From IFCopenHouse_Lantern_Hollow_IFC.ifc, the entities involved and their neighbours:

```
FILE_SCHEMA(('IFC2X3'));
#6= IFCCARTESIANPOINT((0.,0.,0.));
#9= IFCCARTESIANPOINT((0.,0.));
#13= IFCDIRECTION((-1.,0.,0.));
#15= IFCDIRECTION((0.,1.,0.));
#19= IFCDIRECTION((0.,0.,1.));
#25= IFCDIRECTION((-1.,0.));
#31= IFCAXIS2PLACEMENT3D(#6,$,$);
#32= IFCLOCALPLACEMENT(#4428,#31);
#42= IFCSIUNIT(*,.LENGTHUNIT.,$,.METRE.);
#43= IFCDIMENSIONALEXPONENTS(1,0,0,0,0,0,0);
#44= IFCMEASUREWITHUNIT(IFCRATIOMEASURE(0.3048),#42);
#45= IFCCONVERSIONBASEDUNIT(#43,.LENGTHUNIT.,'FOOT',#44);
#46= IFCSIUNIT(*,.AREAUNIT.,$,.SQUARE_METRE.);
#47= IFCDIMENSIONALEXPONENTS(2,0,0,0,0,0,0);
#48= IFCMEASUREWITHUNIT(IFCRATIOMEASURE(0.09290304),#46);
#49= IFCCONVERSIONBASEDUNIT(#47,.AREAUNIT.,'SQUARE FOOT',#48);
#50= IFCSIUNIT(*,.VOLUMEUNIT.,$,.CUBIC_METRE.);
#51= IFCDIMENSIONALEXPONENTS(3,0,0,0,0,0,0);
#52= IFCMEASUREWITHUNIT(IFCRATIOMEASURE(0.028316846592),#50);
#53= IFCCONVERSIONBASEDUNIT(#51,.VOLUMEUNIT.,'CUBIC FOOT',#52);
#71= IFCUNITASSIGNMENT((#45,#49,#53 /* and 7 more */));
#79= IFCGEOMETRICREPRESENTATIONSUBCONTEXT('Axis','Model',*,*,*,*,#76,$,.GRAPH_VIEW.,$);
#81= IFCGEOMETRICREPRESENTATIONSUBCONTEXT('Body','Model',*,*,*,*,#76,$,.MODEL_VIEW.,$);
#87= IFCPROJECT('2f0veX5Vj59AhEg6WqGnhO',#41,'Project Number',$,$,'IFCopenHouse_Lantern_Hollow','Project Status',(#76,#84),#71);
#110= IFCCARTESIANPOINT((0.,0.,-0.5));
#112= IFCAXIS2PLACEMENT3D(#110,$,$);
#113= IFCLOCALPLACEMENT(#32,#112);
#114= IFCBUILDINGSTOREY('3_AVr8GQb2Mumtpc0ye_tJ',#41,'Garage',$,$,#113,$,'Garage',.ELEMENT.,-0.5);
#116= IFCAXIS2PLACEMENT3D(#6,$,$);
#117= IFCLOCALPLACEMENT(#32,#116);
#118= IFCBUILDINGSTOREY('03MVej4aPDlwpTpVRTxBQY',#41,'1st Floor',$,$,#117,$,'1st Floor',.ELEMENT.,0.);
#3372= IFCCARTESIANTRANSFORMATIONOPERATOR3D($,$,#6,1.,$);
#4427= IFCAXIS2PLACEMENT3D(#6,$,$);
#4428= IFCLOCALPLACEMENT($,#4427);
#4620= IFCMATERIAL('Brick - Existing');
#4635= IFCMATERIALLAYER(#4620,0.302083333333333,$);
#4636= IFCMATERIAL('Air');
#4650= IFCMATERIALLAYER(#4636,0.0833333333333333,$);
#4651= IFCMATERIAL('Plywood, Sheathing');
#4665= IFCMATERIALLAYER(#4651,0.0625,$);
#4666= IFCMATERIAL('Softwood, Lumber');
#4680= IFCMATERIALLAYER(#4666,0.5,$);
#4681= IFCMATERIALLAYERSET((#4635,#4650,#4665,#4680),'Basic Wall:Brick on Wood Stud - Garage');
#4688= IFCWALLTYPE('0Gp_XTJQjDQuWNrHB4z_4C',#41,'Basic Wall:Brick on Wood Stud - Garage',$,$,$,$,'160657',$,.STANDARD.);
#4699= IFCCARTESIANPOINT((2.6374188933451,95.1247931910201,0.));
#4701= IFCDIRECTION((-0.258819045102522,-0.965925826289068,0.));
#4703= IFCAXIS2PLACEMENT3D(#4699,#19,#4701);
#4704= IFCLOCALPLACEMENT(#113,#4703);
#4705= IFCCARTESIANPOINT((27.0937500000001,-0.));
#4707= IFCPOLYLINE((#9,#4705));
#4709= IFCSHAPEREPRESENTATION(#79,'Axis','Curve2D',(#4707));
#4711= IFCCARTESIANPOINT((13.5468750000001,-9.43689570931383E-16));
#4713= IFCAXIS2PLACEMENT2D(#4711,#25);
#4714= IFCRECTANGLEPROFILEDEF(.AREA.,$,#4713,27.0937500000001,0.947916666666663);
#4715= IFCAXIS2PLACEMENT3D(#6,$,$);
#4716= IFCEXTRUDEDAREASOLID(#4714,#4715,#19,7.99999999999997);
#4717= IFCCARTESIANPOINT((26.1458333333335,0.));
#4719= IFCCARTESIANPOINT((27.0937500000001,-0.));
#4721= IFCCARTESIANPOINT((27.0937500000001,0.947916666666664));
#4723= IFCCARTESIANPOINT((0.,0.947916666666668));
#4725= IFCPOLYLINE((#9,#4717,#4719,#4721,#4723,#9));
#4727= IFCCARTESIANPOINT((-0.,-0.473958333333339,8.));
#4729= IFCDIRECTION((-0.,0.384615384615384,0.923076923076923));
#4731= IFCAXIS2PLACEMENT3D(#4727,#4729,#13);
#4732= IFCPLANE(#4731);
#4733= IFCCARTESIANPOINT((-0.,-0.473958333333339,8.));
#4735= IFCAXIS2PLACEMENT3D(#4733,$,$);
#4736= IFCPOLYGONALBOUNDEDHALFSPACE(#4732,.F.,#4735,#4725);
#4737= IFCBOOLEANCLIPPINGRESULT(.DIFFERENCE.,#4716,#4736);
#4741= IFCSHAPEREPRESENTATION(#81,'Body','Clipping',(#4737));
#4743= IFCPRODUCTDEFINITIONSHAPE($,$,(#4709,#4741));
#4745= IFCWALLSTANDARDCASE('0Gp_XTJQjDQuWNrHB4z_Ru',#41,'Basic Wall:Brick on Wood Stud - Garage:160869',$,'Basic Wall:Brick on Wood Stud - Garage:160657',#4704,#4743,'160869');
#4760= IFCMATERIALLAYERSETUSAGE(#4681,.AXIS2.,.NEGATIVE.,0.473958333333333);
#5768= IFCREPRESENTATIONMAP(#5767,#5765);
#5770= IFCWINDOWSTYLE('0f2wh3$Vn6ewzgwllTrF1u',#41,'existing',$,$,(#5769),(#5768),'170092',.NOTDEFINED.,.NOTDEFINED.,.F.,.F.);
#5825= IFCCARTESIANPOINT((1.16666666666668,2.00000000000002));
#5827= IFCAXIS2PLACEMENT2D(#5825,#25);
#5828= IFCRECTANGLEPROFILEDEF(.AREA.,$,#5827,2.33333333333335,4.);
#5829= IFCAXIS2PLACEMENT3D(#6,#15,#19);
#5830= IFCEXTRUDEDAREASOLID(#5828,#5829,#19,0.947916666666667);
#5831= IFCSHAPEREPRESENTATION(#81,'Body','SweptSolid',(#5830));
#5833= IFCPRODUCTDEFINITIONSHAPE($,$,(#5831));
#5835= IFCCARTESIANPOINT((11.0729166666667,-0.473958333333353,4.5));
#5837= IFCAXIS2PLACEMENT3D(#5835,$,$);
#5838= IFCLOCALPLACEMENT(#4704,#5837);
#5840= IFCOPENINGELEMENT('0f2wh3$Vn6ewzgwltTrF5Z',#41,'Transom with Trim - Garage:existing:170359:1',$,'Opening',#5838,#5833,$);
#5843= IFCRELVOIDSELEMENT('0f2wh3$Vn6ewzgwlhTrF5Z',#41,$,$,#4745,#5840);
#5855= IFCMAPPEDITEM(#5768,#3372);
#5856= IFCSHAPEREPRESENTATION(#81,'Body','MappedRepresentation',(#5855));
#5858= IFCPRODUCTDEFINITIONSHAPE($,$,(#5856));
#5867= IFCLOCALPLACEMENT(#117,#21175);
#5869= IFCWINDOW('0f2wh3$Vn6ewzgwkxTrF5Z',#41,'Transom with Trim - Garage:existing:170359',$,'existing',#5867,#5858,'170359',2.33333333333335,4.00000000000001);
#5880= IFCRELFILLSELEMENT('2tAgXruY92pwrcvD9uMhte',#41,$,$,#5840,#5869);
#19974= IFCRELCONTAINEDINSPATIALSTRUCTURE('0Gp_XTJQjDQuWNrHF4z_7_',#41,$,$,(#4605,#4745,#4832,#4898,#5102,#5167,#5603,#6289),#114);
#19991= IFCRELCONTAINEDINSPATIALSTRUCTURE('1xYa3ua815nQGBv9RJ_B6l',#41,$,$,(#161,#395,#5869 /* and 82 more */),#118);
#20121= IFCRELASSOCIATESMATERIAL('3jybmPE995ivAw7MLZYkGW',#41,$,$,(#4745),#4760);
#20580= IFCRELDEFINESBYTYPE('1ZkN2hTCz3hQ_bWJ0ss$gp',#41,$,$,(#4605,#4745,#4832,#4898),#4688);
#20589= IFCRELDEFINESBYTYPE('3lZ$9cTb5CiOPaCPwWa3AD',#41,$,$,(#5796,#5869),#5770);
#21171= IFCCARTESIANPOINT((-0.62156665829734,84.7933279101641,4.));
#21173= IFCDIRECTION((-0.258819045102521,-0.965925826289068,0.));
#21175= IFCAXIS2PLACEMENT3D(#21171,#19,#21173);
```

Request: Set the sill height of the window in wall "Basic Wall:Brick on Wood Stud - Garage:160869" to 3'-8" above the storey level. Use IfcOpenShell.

```python
import numpy as np
import ifcopenshell
import ifcopenshell.api.geometry
import ifcopenshell.geom
import ifcopenshell.util.element
import ifcopenshell.util.placement
import ifcopenshell.util.shape
import ifcopenshell.util.unit

model = ifcopenshell.open("IFCopenHouse_Lantern_Hollow_IFC.ifc")
unit_scale = ifcopenshell.util.unit.calculate_unit_scale(model)

window = model.by_id(5869)
opening = window.FillsVoids[0].RelatingOpeningElement
storey = ifcopenshell.util.element.get_container(window, ifc_class="IfcBuildingStorey")
level = ifcopenshell.util.placement.get_local_placement(storey.ObjectPlacement)[2, 3]

# The opening's origin need not be at the sill, so measure its lowest point.
shape = ifcopenshell.geom.create_shape(ifcopenshell.geom.settings(), opening)
bottom = ifcopenshell.util.shape.get_shape_bottom_elevation(shape, shape.geometry) / unit_scale
dz = level + 44 * 0.0254 / unit_scale - bottom

shift = np.array([0.0, 0.0, dz])
# The window is not placed relative to its opening, so move both.
for product in (opening, window):
    matrix = ifcopenshell.util.placement.get_local_placement(product.ObjectPlacement)
    matrix[:3, 3] += shift
    ifcopenshell.api.geometry.edit_object_placement(model, product=product, matrix=matrix, is_si=False)

print(f"moved by {dz * unit_scale:+.3f} m")

model.write("IFCopenHouse_Lantern_Hollow_IFC_rev.ifc")
```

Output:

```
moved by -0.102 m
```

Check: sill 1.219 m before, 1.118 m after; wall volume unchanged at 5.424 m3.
